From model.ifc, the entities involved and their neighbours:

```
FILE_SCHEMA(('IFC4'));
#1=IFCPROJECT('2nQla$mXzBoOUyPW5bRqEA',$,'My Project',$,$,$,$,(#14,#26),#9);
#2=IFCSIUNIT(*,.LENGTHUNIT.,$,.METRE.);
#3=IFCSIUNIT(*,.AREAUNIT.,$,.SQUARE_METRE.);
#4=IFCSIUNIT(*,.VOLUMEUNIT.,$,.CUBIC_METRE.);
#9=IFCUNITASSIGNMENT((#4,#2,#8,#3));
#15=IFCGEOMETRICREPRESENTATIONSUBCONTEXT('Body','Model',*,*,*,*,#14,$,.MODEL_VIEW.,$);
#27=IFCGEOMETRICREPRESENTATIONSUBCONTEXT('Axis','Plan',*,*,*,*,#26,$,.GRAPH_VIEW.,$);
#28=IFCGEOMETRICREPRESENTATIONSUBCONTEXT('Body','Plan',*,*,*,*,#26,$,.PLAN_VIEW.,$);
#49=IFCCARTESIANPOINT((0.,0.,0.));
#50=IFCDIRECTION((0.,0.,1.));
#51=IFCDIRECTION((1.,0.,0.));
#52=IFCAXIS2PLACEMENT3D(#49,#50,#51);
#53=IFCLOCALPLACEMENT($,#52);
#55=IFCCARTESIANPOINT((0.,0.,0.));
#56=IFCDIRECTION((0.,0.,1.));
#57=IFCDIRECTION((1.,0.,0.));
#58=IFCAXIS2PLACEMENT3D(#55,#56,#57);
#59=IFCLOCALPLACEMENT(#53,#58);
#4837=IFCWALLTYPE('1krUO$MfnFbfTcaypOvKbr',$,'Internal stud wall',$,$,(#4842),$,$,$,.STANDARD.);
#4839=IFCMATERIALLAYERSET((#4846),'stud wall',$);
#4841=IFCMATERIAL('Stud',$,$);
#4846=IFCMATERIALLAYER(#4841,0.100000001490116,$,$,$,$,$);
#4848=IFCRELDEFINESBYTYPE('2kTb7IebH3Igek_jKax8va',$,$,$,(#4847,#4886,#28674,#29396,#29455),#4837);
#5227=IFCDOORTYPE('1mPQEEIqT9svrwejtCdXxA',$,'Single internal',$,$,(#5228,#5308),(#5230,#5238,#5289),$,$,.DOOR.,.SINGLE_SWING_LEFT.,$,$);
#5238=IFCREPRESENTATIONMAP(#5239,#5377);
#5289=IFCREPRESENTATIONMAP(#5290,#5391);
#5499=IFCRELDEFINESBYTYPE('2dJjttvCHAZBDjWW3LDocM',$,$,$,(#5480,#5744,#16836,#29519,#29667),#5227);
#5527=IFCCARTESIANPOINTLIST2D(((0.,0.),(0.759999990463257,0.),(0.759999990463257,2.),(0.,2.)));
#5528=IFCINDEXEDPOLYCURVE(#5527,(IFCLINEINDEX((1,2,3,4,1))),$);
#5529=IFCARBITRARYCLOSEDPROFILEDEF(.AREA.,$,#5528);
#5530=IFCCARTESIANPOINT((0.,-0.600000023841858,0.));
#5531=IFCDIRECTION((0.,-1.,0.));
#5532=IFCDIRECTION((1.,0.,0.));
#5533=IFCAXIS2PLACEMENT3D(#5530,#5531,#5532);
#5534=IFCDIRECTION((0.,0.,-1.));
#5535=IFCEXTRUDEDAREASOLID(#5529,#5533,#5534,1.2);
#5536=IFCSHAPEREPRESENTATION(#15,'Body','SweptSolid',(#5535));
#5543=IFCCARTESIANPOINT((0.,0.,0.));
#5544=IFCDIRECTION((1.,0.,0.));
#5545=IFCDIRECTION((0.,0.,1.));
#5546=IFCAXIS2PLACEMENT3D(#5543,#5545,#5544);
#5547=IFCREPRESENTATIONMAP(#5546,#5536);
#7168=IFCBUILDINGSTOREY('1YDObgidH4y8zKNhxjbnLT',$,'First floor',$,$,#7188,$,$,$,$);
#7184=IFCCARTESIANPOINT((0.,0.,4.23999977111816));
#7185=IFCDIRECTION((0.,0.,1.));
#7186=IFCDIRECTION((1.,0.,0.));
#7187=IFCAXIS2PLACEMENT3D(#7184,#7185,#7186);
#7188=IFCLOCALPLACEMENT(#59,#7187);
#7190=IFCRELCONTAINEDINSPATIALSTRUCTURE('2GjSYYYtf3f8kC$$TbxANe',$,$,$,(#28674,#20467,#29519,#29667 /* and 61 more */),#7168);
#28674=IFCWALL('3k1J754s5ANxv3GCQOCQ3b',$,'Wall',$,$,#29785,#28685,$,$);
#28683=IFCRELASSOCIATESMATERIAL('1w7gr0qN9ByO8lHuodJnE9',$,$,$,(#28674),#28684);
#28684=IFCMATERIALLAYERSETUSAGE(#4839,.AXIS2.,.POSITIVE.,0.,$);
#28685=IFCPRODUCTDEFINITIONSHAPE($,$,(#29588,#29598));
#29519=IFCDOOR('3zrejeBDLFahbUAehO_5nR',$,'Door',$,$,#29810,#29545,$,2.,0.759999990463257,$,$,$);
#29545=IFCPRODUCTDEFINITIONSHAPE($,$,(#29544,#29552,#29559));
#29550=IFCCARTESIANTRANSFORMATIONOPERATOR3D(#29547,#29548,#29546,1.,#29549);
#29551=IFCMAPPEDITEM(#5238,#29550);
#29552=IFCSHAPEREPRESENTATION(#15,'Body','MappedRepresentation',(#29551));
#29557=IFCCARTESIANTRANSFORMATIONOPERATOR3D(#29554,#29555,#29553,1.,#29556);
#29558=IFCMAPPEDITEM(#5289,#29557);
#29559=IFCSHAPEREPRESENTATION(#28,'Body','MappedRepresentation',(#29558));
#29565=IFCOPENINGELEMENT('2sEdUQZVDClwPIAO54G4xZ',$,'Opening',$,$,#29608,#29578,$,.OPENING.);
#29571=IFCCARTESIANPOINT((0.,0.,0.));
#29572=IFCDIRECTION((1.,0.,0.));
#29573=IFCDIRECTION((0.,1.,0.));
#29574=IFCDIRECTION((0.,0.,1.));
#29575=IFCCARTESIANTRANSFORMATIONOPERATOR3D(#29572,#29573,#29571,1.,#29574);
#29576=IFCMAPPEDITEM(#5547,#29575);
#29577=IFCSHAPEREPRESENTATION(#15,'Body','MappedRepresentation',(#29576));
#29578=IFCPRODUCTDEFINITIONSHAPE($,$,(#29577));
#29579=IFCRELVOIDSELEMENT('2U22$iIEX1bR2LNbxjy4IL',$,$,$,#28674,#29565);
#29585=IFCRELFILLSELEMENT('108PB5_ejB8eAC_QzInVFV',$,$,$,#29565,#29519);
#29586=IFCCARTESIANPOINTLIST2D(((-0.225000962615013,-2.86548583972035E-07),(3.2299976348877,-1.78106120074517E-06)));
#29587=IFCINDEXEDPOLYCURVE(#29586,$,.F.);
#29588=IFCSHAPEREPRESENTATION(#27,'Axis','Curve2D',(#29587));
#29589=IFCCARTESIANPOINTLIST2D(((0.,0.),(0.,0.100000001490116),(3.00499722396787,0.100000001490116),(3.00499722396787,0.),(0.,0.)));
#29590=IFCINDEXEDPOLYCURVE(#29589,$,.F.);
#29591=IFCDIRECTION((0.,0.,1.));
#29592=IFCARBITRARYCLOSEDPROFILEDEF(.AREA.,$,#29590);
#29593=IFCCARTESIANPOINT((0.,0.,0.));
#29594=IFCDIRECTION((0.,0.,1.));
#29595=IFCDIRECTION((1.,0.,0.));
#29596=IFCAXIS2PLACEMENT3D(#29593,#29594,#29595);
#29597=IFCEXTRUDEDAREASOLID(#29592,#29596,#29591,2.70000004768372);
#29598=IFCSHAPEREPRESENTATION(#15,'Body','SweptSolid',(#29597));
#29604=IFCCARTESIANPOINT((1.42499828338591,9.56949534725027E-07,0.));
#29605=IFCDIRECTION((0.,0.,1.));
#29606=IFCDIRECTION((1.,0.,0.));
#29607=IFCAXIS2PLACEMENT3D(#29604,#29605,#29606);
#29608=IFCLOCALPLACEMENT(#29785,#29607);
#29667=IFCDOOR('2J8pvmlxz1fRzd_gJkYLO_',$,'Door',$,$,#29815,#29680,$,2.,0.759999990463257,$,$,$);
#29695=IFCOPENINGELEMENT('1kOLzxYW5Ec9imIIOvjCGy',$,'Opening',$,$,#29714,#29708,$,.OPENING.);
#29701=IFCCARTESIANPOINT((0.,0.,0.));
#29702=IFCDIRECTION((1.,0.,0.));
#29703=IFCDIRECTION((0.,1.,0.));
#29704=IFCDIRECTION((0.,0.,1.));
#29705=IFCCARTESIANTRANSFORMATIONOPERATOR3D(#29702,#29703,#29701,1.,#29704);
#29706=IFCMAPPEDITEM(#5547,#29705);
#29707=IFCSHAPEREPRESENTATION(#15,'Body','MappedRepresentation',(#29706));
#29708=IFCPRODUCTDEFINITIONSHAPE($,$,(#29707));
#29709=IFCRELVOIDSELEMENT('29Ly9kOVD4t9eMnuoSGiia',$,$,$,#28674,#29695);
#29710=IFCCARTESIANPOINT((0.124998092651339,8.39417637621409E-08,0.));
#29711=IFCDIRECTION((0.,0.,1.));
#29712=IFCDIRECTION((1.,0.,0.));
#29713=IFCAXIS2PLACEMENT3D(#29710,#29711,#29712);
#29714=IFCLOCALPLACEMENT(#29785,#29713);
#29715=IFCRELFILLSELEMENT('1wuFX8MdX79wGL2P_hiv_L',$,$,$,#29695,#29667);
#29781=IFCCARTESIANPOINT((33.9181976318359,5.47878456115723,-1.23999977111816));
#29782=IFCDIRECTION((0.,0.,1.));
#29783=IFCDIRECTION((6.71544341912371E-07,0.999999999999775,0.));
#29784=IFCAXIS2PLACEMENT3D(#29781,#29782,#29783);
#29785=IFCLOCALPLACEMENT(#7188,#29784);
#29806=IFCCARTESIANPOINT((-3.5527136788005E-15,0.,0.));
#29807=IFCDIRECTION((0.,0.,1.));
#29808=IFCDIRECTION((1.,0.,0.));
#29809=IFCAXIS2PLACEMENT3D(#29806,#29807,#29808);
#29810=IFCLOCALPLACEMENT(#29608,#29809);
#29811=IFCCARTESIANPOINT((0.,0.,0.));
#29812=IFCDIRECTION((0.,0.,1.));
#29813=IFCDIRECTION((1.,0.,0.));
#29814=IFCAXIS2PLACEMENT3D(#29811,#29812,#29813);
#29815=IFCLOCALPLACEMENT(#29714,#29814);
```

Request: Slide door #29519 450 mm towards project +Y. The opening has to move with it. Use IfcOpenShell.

```python
import ifcopenshell
import ifcopenshell.api.geometry
import ifcopenshell.util.placement

model = ifcopenshell.open("model.ifc")

door = model.by_guid("3zrejeBDLFahbUAehO_5nR")
opening = door.FillsVoids[0].RelatingOpeningElement
wall = opening.VoidsElements[0].RelatingBuildingElement

wall_matrix = ifcopenshell.util.placement.get_local_placement(wall.ObjectPlacement)
shift = wall_matrix[:3, 0] * 0.45
before = ifcopenshell.util.placement.get_local_placement(door.ObjectPlacement)[:3, 3].copy()

# The door is placed relative to its opening, so it follows when the opening moves.
matrix = ifcopenshell.util.placement.get_local_placement(opening.ObjectPlacement)
matrix[:3, 3] += shift
ifcopenshell.api.geometry.edit_object_placement(
    model, product=opening, matrix=matrix, is_si=False, should_transform_children=True
)

after = ifcopenshell.util.placement.get_local_placement(door.ObjectPlacement)[:3, 3]
print("door moved by", (after - before).round(3) + 0.0)

model.write("model-out.ifc")
```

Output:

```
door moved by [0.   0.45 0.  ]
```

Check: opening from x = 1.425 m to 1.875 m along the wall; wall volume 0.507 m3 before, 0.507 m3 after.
